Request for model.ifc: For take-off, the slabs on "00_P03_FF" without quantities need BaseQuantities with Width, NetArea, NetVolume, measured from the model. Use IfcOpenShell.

First a look at what the model holds.

```python
import ifcopenshell
import ifcopenshell.util.element
import ifcopenshell.util.unit

model = ifcopenshell.open("model.ifc")
print(model.schema)
for unit_type in ("LENGTHUNIT", "AREAUNIT", "VOLUMEUNIT"):
    print(unit_type, ifcopenshell.util.unit.calculate_unit_scale(model, unit_type))
storey = next(s for s in model.by_type("IfcBuildingStorey") if s.Name == "00_P03_FF")
slabs = [e for e in ifcopenshell.util.element.get_decomposition(storey) if e.is_a("IfcSlab")]
for e in sorted(slabs, key=lambda e: e.id()):
    print(e.id(), e.is_a(), e.Name, list(ifcopenshell.util.element.get_psets(e, qtos_only=True)), sep=" | ")
```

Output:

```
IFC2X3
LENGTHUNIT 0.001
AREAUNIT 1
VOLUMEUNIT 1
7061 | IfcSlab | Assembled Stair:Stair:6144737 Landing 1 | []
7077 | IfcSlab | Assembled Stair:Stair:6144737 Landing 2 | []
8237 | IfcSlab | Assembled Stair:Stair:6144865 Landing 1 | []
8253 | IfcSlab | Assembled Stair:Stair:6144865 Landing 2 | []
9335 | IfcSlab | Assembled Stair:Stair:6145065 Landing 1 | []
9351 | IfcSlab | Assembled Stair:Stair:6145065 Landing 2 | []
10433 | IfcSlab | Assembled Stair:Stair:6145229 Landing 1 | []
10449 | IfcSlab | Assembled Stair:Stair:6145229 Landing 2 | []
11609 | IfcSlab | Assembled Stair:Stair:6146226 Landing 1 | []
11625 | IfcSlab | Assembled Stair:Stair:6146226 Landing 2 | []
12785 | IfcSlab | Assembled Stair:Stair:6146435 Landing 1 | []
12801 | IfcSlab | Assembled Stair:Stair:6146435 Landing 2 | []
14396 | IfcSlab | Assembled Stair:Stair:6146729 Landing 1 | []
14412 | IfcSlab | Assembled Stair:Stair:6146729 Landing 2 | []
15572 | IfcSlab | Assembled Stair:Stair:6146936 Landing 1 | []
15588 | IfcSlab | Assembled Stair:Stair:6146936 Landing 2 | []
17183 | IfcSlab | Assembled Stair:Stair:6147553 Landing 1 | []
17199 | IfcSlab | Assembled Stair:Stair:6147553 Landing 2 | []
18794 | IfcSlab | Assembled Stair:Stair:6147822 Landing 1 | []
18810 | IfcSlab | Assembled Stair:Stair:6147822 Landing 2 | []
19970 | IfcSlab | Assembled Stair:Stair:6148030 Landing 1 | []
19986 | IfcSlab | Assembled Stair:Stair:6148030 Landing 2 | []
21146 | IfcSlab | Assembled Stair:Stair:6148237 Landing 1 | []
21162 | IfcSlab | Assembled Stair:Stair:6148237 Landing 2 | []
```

```python
import ifcopenshell
import ifcopenshell.api.pset
import ifcopenshell.geom
import ifcopenshell.util.element
import ifcopenshell.util.shape
import ifcopenshell.util.unit

model = ifcopenshell.open("model.ifc")
unit_scale = ifcopenshell.util.unit.calculate_unit_scale(model)
area_scale = ifcopenshell.util.unit.calculate_unit_scale(model, "AREAUNIT")
volume_scale = ifcopenshell.util.unit.calculate_unit_scale(model, "VOLUMEUNIT")
settings = ifcopenshell.geom.settings()

storey = next(s for s in model.by_type("IfcBuildingStorey") if s.Name == "00_P03_FF")
slabs = [e for e in ifcopenshell.util.element.get_decomposition(storey) if e.is_a("IfcSlab")]

for e in sorted(slabs, key=lambda e: e.id()):
    if ifcopenshell.util.element.get_psets(e, qtos_only=True, should_inherit=False):
        continue
    # Geometry comes back in metres, in the element's own axes.
    shape = ifcopenshell.geom.create_shape(settings, e)
    values = {
        "Width": ifcopenshell.util.shape.get_z(shape.geometry) / unit_scale,
        "NetArea": ifcopenshell.util.shape.get_footprint_area(shape.geometry) / area_scale,
        "NetVolume": ifcopenshell.util.shape.get_volume(shape.geometry) / volume_scale,
    }
    qto = ifcopenshell.api.pset.add_qto(model, product=e, name="BaseQuantities")
    ifcopenshell.api.pset.edit_qto(model, qto=qto, properties=values)
    print(e.id(), {k: round(v, 3) for k, v in values.items()})

model.write("model_updated.ifc")
```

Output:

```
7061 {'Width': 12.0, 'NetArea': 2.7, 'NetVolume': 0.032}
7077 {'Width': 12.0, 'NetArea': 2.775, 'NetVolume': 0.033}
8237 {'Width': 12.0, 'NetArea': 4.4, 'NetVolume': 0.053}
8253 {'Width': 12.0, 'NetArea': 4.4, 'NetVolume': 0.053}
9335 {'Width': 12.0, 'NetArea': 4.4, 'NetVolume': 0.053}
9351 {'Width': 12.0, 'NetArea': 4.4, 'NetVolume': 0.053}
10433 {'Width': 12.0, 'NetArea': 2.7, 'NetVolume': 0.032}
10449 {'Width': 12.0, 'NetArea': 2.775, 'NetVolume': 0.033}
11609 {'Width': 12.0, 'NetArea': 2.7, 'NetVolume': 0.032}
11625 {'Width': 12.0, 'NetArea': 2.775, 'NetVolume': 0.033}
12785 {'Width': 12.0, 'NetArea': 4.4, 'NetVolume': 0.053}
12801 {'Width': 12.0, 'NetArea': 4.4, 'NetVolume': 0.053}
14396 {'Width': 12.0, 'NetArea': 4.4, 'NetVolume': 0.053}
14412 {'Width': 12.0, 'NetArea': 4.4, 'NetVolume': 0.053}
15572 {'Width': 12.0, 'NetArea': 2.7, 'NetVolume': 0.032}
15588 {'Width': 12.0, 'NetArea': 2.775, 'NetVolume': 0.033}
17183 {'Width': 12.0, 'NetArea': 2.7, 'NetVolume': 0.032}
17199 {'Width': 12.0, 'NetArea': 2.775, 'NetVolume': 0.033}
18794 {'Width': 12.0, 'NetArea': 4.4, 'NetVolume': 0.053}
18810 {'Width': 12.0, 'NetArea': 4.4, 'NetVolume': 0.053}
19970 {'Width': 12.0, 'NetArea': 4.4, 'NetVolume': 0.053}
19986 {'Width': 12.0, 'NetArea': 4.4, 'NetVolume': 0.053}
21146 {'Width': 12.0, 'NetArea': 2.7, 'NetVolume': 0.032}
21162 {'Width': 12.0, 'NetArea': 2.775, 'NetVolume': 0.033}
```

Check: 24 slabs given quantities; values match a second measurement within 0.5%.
